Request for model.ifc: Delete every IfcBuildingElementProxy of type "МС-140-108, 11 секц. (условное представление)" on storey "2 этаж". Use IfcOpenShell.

First a look at what the model holds.

```python
import ifcopenshell
import ifcopenshell.util.element

model = ifcopenshell.open("model.ifc")
print(model.schema)
storey = next(s for s in model.by_type("IfcBuildingStorey") if s.Name == "2 этаж")
proxies = [e for e in ifcopenshell.util.element.get_decomposition(storey) if e.is_a("IfcBuildingElementProxy")]
seen = {}
for e in proxies:
    element_type = ifcopenshell.util.element.get_type(e)
    name = element_type.Name if element_type not in (None, e) else None
    seen[name] = seen.get(name, 0) + 1
for name, count in sorted(seen.items(), key=str):
    print(count, "x", name)
```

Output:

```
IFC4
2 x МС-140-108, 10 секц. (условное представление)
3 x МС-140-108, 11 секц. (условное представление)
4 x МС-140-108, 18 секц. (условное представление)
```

```python
import ifcopenshell
import ifcopenshell.api.root
import ifcopenshell.util.element

model = ifcopenshell.open("model.ifc")

storey = next(s for s in model.by_type("IfcBuildingStorey") if s.Name == "2 этаж")
proxies = [e for e in ifcopenshell.util.element.get_decomposition(storey) if e.is_a("IfcBuildingElementProxy")]
targets = [e for e in proxies if (t := ifcopenshell.util.element.get_type(e)) not in (None, e) and t.Name == "МС-140-108, 11 секц. (условное представление)"]

for e in targets:
    ifcopenshell.api.root.remove_product(model, product=e)
print(len(targets), "removed")

model.write("model_updated.ifc")
```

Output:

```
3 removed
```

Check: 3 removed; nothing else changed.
